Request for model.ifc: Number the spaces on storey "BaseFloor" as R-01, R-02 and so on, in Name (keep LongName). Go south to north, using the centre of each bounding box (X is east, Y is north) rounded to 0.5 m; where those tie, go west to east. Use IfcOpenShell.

First a look at what the model holds.

```python
import ifcopenshell
import ifcopenshell.util.element
import ifcopenshell.util.placement

model = ifcopenshell.open("model.ifc")
print(model.schema)
storey = next(s for s in model.by_type("IfcBuildingStorey") if s.Name == "BaseFloor")
spaces = [e for e in ifcopenshell.util.element.get_decomposition(storey) if e.is_a("IfcSpace")]
for e in sorted(spaces, key=lambda e: e.id()):
    origin = ifcopenshell.util.placement.get_local_placement(e.ObjectPlacement)[:3, 3]
    print(e.id(), e.Name, e.LongName, origin.round(2) + 0.0, sep=" | ")
```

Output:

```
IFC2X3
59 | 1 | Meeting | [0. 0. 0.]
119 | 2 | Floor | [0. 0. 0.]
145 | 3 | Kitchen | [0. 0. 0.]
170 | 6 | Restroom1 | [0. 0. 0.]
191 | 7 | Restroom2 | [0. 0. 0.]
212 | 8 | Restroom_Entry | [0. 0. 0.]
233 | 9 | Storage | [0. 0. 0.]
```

```python
import ifcopenshell
import ifcopenshell.geom
import ifcopenshell.util.element
import ifcopenshell.util.shape

model = ifcopenshell.open("model.ifc")
settings = ifcopenshell.geom.settings()
settings.set("use-world-coords", True)


def centre(element):
    shape = ifcopenshell.geom.create_shape(settings, element)
    return ifcopenshell.util.shape.get_bbox_centroid(shape.geometry)


storey = next(s for s in model.by_type("IfcBuildingStorey") if s.Name == "BaseFloor")
spaces = [e for e in ifcopenshell.util.element.get_decomposition(storey) if e.is_a("IfcSpace")]

# Insertion points can sit at a corner or the storey origin, so sort by the geometry (in metres).
centres = {e: centre(e) for e in spaces}
spaces.sort(key=lambda e: (round(centres[e][1] / 0.5), centres[e][0]))

for i, e in enumerate(spaces, start=1):
    number = f"R-{i:02d}"
    e.Name = number
    print(e.id(), number)

model.write("model_v2.ifc")
```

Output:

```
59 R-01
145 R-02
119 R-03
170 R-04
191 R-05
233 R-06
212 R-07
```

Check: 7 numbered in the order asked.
